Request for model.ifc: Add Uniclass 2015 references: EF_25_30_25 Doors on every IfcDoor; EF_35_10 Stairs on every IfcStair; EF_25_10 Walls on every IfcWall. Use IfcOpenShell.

First a look at what the model holds.

```python
import ifcopenshell

model = ifcopenshell.open("model.ifc")
print(model.schema)
print("classifications:", [c.Name for c in model.by_type("IfcClassification")])
for ifc_class in ("IfcDoor", "IfcRoof", "IfcStair", "IfcWall", "IfcWindow"):
    print(ifc_class, len(model.by_type(ifc_class)))
```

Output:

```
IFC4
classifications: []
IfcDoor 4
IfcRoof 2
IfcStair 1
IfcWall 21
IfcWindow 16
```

```python
import ifcopenshell
import ifcopenshell.api.classification

model = ifcopenshell.open("model.ifc")

system = ifcopenshell.api.classification.add_classification(model, classification="Uniclass 2015")

codes = {
    "IfcDoor": ("EF_25_30_25", "Doors"),
    "IfcStair": ("EF_35_10", "Stairs"),
    "IfcWall": ("EF_25_10", "Walls"),
}
for ifc_class, (code, name) in codes.items():
    products = model.by_type(ifc_class)
    ifcopenshell.api.classification.add_reference(
        model, products=products, classification=system, identification=code, name=name
    )
    print(code, len(products))

model.write("model_v2.ifc")
```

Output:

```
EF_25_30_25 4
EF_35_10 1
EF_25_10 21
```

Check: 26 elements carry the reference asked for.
